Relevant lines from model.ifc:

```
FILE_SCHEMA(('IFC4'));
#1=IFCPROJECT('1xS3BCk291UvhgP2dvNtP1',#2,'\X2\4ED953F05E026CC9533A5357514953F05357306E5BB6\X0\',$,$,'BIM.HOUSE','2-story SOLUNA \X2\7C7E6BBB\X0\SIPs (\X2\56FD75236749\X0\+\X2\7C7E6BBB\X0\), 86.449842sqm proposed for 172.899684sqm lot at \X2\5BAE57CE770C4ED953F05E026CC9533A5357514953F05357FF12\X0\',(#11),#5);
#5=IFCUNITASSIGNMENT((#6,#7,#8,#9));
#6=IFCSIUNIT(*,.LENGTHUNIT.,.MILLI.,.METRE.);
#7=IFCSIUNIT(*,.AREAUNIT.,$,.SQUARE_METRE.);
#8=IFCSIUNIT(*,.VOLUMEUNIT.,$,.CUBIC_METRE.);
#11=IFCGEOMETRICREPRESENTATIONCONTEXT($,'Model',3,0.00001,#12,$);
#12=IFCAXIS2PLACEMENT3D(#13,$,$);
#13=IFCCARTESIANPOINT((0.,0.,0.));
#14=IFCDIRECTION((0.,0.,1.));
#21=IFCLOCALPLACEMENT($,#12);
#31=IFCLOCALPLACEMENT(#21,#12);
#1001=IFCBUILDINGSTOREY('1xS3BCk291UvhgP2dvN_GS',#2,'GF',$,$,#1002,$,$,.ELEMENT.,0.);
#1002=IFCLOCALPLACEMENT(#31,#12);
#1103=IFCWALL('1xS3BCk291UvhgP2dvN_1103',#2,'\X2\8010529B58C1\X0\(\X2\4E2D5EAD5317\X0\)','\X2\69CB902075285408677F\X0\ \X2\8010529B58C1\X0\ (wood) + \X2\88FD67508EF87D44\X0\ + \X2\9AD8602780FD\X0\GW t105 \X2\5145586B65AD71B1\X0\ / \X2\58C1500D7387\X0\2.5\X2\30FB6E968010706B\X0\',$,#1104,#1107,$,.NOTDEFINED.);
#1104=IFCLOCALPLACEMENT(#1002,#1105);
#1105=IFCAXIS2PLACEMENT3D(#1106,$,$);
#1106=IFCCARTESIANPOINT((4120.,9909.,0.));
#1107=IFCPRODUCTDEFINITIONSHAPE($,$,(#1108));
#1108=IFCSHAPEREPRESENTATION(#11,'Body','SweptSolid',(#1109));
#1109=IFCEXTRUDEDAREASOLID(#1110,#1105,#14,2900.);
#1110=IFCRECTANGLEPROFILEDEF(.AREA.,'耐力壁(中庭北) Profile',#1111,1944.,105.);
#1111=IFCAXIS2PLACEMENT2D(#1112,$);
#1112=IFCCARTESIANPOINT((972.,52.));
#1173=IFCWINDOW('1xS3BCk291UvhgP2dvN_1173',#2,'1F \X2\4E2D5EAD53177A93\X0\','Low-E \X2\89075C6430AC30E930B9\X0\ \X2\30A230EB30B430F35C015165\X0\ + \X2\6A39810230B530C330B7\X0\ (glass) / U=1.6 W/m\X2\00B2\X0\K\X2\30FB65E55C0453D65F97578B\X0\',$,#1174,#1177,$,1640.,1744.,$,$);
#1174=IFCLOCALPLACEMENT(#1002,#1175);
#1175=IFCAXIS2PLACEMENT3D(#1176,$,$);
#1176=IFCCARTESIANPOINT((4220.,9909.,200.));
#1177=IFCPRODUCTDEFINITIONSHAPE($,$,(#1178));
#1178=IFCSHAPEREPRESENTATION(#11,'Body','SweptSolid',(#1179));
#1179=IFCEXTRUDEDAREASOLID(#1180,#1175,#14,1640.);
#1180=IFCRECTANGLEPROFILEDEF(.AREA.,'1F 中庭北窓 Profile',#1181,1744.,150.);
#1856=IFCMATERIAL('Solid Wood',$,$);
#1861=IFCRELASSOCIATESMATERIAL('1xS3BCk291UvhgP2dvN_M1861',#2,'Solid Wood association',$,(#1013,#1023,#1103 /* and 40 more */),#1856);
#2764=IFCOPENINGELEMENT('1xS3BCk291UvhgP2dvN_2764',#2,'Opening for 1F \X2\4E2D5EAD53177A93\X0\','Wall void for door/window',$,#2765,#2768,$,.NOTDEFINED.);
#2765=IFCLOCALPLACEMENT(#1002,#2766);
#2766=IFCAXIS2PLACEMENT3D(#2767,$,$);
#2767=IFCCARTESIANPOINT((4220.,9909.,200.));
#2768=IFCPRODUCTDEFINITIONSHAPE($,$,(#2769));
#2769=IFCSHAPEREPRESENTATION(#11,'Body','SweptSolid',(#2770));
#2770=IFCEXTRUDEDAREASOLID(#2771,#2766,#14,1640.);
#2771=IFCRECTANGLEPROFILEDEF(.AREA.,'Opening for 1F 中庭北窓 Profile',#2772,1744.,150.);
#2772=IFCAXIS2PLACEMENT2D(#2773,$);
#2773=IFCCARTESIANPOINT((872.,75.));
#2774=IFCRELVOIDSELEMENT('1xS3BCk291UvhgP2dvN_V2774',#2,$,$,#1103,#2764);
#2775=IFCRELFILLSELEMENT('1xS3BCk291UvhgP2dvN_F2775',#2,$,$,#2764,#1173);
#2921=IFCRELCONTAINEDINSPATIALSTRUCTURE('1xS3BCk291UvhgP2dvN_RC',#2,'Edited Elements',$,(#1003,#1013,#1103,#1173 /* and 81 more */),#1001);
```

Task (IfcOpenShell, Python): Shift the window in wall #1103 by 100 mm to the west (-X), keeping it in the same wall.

```python
import ifcopenshell
import ifcopenshell.api.geometry
import ifcopenshell.util.placement
import ifcopenshell.util.unit

model = ifcopenshell.open("model.ifc")
unit_scale = ifcopenshell.util.unit.calculate_unit_scale(model)

window = model.by_guid("1xS3BCk291UvhgP2dvN_1173")
opening = window.FillsVoids[0].RelatingOpeningElement
wall = opening.VoidsElements[0].RelatingBuildingElement

wall_matrix = ifcopenshell.util.placement.get_local_placement(wall.ObjectPlacement)
shift = wall_matrix[:3, 0] * -0.1 / unit_scale
before = ifcopenshell.util.placement.get_local_placement(window.ObjectPlacement)[:3, 3].copy()

# The window is not placed relative to its opening, so move both.
for product in (opening, window):
    matrix = ifcopenshell.util.placement.get_local_placement(product.ObjectPlacement)
    matrix[:3, 3] += shift
    ifcopenshell.api.geometry.edit_object_placement(model, product=product, matrix=matrix, is_si=False)

after = ifcopenshell.util.placement.get_local_placement(window.ObjectPlacement)[:3, 3]
print("window moved by", (after - before).round(3) + 0.0)

model.write("model-out.ifc")
```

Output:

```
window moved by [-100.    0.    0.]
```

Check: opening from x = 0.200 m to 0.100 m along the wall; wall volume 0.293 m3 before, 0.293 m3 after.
